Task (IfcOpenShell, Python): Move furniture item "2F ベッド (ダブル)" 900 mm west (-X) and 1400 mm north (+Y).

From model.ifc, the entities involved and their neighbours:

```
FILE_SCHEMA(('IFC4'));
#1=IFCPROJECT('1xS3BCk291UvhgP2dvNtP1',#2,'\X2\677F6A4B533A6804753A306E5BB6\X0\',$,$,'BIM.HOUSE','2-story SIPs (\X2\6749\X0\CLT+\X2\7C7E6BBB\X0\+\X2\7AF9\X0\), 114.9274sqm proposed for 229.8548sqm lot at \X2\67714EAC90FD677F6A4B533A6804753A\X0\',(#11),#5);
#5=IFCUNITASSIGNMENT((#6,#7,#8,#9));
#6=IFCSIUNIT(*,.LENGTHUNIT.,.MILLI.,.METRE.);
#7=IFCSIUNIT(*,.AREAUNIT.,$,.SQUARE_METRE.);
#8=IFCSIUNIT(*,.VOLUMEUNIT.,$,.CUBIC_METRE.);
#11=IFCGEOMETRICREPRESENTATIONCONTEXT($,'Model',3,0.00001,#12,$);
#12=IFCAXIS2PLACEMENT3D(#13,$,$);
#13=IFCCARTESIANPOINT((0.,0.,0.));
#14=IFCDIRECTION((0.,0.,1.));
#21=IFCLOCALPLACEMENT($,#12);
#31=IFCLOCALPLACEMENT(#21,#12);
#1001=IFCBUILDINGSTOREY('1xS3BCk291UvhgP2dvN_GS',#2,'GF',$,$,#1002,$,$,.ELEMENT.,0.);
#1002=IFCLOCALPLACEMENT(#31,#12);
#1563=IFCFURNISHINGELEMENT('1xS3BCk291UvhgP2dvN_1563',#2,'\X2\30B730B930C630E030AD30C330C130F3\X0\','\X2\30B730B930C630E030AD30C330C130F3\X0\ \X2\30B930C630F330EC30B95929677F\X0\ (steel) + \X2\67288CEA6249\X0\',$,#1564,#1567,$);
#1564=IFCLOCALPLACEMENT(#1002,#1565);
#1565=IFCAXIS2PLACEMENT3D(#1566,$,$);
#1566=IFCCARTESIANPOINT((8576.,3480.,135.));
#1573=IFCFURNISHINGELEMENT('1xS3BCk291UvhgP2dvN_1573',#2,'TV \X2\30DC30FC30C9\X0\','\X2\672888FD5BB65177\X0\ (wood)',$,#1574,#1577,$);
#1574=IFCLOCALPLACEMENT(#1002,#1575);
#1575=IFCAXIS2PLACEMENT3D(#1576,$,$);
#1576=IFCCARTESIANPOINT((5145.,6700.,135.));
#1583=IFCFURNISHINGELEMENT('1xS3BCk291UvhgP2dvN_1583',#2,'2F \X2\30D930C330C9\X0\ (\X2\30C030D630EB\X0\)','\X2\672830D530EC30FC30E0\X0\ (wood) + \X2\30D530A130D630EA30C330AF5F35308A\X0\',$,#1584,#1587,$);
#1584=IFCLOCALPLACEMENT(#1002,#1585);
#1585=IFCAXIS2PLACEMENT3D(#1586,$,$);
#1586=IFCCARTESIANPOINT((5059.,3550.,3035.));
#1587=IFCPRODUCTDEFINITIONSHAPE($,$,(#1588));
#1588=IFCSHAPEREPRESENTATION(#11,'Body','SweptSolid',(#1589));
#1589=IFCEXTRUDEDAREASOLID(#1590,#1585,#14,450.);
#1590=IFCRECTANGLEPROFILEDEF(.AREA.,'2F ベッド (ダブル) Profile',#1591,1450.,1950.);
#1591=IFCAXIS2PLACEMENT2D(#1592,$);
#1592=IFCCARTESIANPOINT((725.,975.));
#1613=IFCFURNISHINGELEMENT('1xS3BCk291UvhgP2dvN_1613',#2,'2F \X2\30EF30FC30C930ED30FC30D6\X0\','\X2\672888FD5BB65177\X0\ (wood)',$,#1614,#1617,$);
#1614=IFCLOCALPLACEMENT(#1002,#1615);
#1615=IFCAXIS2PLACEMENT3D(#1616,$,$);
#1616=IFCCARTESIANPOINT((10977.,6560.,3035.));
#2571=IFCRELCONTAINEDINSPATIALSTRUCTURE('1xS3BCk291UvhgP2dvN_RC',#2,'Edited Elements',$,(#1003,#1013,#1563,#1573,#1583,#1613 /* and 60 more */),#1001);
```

```python
import ifcopenshell
import ifcopenshell.api.geometry
import ifcopenshell.util.placement
import ifcopenshell.util.unit

model = ifcopenshell.open("model.ifc")
unit_scale = ifcopenshell.util.unit.calculate_unit_scale(model)

item = model.by_guid("1xS3BCk291UvhgP2dvN_1583")
matrix = ifcopenshell.util.placement.get_local_placement(item.ObjectPlacement)
matrix[0, 3] -= 0.9 / unit_scale
matrix[1, 3] += 1.4 / unit_scale
ifcopenshell.api.geometry.edit_object_placement(model, product=item, matrix=matrix, is_si=False)

print(ifcopenshell.util.placement.get_local_placement(item.ObjectPlacement).round(3) + 0.0)

model.write("model_rev.ifc")
```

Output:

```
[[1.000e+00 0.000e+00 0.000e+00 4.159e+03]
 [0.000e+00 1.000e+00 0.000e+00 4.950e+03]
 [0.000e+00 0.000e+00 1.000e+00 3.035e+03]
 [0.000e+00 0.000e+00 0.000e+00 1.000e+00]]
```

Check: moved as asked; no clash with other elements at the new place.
